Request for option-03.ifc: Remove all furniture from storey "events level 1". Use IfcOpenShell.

First a look at what the model holds.

```python
import ifcopenshell
import ifcopenshell.util.element

model = ifcopenshell.open("option-03.ifc")
print(model.schema)
storey = next(s for s in model.by_type("IfcBuildingStorey") if s.Name == "events level 1")
furniture = [e for e in ifcopenshell.util.element.get_decomposition(storey) if e.is_a("IfcFurnishingElement")]
seen = {}
for e in furniture:
    element_type = ifcopenshell.util.element.get_type(e)
    name = element_type.Name if element_type not in (None, e) else None
    seen[name] = seen.get(name, 0) + 1
for name, count in sorted(seen.items(), key=str):
    print(count, "x", name)
```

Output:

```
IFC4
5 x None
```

```python
import ifcopenshell
import ifcopenshell.api.root
import ifcopenshell.util.element

model = ifcopenshell.open("option-03.ifc")

storey = next(s for s in model.by_type("IfcBuildingStorey") if s.Name == "events level 1")
furniture = [e for e in ifcopenshell.util.element.get_decomposition(storey) if e.is_a("IfcFurnishingElement")]

for e in furniture:
    ifcopenshell.api.root.remove_product(model, product=e)
print(len(furniture), "removed")

model.write("option-03-out.ifc")
```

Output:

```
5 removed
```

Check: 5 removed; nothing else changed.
